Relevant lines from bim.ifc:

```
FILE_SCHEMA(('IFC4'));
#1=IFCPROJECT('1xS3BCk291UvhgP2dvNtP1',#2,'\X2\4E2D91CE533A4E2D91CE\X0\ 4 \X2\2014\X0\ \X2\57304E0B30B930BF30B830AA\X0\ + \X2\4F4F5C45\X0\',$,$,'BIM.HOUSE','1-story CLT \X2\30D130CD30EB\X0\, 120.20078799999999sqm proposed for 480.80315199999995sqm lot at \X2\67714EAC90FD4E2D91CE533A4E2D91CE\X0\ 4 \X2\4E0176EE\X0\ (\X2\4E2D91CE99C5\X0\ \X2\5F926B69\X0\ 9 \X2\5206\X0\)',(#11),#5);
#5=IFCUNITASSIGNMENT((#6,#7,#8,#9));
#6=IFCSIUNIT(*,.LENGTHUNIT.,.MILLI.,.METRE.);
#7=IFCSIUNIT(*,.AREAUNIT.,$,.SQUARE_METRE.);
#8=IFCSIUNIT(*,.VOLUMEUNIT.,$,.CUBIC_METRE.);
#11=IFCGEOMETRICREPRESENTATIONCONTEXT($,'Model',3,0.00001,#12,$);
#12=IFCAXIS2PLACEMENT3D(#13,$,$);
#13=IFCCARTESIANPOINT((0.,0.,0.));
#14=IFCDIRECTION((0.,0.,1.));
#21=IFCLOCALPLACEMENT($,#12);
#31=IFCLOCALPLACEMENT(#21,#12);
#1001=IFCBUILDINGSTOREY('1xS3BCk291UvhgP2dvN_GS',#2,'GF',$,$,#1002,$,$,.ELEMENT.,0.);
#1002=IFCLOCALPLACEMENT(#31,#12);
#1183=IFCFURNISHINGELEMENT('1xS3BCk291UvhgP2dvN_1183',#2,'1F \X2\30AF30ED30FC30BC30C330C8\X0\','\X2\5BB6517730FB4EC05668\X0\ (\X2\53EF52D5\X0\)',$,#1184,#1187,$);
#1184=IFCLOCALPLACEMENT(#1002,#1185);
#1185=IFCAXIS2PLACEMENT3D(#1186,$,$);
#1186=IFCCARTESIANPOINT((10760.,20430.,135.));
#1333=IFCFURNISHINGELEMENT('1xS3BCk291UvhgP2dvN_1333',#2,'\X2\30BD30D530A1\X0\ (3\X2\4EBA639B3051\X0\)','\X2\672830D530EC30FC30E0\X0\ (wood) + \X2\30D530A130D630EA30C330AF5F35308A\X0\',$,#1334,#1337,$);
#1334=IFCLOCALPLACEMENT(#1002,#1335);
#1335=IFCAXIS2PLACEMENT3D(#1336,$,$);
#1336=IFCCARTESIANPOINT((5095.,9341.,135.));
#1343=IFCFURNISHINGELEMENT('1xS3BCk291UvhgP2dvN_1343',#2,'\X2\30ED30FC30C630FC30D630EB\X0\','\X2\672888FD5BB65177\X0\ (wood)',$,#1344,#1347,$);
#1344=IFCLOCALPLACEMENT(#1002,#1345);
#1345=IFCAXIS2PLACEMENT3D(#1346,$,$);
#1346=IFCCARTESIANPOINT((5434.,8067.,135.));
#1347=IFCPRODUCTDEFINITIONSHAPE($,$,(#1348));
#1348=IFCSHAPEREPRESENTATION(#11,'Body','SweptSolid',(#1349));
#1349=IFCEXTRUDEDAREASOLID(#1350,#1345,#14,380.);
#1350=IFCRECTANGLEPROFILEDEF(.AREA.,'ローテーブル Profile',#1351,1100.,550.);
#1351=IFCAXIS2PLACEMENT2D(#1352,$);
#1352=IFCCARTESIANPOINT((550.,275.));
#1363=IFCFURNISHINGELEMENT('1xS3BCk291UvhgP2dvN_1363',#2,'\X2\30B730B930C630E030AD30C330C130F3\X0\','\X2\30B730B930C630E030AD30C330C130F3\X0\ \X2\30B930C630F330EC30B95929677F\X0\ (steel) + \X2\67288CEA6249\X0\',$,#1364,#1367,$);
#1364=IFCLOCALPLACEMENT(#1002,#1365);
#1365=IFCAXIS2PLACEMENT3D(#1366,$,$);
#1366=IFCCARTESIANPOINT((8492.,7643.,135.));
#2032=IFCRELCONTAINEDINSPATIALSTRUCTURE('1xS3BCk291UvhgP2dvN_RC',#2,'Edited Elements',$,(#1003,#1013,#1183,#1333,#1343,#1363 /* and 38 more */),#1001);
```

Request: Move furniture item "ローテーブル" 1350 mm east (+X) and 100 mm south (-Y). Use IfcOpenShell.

```python
import ifcopenshell
import ifcopenshell.api.geometry
import ifcopenshell.util.placement
import ifcopenshell.util.unit

model = ifcopenshell.open("bim.ifc")
unit_scale = ifcopenshell.util.unit.calculate_unit_scale(model)

item = model.by_guid("1xS3BCk291UvhgP2dvN_1343")
matrix = ifcopenshell.util.placement.get_local_placement(item.ObjectPlacement)
matrix[0, 3] += 1.35 / unit_scale
matrix[1, 3] -= 0.1 / unit_scale
ifcopenshell.api.geometry.edit_object_placement(model, product=item, matrix=matrix, is_si=False)

print(ifcopenshell.util.placement.get_local_placement(item.ObjectPlacement).round(3) + 0.0)

model.write("bim_updated.ifc")
```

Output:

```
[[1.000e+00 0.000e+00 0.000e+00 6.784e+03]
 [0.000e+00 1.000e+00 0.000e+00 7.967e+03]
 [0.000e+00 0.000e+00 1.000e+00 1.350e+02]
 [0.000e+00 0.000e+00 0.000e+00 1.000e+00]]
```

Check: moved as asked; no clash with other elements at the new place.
